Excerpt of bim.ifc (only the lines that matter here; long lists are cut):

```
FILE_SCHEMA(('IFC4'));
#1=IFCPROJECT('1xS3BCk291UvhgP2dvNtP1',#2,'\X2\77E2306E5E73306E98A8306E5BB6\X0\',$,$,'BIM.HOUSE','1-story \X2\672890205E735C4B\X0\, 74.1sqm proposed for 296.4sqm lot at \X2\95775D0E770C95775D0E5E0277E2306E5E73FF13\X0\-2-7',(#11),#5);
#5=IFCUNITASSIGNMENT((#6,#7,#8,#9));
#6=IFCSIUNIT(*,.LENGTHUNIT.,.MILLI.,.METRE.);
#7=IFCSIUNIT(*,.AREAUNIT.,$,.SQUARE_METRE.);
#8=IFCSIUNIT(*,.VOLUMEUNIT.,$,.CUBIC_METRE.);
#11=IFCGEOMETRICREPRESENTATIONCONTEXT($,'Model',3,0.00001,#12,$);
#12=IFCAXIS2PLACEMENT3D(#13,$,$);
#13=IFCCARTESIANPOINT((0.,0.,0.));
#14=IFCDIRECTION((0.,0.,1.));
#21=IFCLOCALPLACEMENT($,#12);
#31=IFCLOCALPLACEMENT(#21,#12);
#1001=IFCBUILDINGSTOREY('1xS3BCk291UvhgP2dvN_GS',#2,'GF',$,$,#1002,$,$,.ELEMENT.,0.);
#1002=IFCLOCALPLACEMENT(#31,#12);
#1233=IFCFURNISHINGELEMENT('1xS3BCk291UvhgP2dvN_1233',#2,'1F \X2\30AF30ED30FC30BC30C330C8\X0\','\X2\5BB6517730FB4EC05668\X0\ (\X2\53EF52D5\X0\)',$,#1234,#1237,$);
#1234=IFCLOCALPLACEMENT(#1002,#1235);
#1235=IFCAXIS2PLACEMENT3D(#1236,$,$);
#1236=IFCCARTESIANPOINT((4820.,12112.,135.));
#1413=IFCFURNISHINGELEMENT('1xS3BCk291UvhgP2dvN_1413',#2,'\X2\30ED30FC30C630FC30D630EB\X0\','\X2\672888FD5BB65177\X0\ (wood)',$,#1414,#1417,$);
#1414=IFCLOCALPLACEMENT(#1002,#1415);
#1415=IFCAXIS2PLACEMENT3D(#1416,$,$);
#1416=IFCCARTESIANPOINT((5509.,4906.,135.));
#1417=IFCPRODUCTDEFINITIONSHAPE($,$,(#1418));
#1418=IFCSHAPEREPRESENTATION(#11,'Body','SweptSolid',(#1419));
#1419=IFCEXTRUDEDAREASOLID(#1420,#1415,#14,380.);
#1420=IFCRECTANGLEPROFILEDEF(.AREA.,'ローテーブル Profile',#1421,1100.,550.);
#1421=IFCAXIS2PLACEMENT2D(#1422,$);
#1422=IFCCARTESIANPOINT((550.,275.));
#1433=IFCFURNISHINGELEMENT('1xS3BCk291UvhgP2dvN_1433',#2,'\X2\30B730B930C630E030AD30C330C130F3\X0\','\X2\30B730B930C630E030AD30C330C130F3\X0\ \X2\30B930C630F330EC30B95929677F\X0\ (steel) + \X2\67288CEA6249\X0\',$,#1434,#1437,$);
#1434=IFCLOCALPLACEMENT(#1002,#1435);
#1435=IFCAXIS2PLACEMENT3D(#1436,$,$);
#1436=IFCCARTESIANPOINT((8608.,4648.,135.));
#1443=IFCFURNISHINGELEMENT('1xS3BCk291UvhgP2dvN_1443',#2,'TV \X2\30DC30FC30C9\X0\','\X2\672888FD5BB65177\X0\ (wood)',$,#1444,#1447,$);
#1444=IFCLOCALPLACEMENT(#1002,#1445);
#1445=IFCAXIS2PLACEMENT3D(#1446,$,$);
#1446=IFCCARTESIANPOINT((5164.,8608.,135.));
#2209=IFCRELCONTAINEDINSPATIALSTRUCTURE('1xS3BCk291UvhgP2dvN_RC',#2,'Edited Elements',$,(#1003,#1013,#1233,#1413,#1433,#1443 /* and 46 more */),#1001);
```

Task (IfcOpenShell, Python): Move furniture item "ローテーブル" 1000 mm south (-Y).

```python
import ifcopenshell
import ifcopenshell.api.geometry
import ifcopenshell.util.placement

model = ifcopenshell.open("bim.ifc")

item = model.by_id(1413)
matrix = ifcopenshell.util.placement.get_local_placement(item.ObjectPlacement)
matrix[1, 3] -= 1000.0
ifcopenshell.api.geometry.edit_object_placement(model, product=item, matrix=matrix, is_si=False)

print(ifcopenshell.util.placement.get_local_placement(item.ObjectPlacement).round(3) + 0.0)

model.write("bim_updated.ifc")
```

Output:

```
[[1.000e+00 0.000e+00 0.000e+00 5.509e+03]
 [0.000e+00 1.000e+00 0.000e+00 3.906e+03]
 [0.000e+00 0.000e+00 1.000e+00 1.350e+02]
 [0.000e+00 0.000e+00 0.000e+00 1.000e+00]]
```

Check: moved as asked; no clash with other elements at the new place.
